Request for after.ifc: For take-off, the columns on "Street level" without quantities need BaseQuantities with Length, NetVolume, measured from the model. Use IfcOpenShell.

First a look at what the model holds.

```python
import ifcopenshell
import ifcopenshell.util.element
import ifcopenshell.util.unit

model = ifcopenshell.open("after.ifc")
print(model.schema)
for unit_type in ("LENGTHUNIT", "AREAUNIT", "VOLUMEUNIT"):
    print(unit_type, ifcopenshell.util.unit.calculate_unit_scale(model, unit_type))
storey = next(s for s in model.by_type("IfcBuildingStorey") if s.Name == "Street level")
columns = [e for e in ifcopenshell.util.element.get_decomposition(storey) if e.is_a("IfcColumn")]
for e in sorted(columns, key=lambda e: e.id()):
    print(e.id(), e.is_a(), e.Name, list(ifcopenshell.util.element.get_psets(e, qtos_only=True)), sep=" | ")
```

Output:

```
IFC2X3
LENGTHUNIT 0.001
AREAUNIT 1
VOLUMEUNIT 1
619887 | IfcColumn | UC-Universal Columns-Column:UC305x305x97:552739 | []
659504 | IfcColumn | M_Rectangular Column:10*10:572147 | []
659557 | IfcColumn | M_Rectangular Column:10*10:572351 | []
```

```python
import ifcopenshell
import ifcopenshell.api.pset
import ifcopenshell.geom
import ifcopenshell.util.element
import ifcopenshell.util.shape
import ifcopenshell.util.unit

model = ifcopenshell.open("after.ifc")
unit_scale = ifcopenshell.util.unit.calculate_unit_scale(model)
volume_scale = ifcopenshell.util.unit.calculate_unit_scale(model, "VOLUMEUNIT")
settings = ifcopenshell.geom.settings()

storey = next(s for s in model.by_type("IfcBuildingStorey") if s.Name == "Street level")
columns = [e for e in ifcopenshell.util.element.get_decomposition(storey) if e.is_a("IfcColumn")]

for e in sorted(columns, key=lambda e: e.id()):
    if ifcopenshell.util.element.get_psets(e, qtos_only=True, should_inherit=False):
        continue
    # Geometry comes back in metres, in the element's own axes.
    shape = ifcopenshell.geom.create_shape(settings, e)
    values = {
        "Length": ifcopenshell.util.shape.get_z(shape.geometry) / unit_scale,
        "NetVolume": ifcopenshell.util.shape.get_volume(shape.geometry) / volume_scale,
    }
    qto = ifcopenshell.api.pset.add_qto(model, product=e, name="BaseQuantities")
    ifcopenshell.api.pset.edit_qto(model, qto=qto, properties=values)
    print(e.id(), {k: round(v, 3) for k, v in values.items()})

model.write("after_edited.ifc")
```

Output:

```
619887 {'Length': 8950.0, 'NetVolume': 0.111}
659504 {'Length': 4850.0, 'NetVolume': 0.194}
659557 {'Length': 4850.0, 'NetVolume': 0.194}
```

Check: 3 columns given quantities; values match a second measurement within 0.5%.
